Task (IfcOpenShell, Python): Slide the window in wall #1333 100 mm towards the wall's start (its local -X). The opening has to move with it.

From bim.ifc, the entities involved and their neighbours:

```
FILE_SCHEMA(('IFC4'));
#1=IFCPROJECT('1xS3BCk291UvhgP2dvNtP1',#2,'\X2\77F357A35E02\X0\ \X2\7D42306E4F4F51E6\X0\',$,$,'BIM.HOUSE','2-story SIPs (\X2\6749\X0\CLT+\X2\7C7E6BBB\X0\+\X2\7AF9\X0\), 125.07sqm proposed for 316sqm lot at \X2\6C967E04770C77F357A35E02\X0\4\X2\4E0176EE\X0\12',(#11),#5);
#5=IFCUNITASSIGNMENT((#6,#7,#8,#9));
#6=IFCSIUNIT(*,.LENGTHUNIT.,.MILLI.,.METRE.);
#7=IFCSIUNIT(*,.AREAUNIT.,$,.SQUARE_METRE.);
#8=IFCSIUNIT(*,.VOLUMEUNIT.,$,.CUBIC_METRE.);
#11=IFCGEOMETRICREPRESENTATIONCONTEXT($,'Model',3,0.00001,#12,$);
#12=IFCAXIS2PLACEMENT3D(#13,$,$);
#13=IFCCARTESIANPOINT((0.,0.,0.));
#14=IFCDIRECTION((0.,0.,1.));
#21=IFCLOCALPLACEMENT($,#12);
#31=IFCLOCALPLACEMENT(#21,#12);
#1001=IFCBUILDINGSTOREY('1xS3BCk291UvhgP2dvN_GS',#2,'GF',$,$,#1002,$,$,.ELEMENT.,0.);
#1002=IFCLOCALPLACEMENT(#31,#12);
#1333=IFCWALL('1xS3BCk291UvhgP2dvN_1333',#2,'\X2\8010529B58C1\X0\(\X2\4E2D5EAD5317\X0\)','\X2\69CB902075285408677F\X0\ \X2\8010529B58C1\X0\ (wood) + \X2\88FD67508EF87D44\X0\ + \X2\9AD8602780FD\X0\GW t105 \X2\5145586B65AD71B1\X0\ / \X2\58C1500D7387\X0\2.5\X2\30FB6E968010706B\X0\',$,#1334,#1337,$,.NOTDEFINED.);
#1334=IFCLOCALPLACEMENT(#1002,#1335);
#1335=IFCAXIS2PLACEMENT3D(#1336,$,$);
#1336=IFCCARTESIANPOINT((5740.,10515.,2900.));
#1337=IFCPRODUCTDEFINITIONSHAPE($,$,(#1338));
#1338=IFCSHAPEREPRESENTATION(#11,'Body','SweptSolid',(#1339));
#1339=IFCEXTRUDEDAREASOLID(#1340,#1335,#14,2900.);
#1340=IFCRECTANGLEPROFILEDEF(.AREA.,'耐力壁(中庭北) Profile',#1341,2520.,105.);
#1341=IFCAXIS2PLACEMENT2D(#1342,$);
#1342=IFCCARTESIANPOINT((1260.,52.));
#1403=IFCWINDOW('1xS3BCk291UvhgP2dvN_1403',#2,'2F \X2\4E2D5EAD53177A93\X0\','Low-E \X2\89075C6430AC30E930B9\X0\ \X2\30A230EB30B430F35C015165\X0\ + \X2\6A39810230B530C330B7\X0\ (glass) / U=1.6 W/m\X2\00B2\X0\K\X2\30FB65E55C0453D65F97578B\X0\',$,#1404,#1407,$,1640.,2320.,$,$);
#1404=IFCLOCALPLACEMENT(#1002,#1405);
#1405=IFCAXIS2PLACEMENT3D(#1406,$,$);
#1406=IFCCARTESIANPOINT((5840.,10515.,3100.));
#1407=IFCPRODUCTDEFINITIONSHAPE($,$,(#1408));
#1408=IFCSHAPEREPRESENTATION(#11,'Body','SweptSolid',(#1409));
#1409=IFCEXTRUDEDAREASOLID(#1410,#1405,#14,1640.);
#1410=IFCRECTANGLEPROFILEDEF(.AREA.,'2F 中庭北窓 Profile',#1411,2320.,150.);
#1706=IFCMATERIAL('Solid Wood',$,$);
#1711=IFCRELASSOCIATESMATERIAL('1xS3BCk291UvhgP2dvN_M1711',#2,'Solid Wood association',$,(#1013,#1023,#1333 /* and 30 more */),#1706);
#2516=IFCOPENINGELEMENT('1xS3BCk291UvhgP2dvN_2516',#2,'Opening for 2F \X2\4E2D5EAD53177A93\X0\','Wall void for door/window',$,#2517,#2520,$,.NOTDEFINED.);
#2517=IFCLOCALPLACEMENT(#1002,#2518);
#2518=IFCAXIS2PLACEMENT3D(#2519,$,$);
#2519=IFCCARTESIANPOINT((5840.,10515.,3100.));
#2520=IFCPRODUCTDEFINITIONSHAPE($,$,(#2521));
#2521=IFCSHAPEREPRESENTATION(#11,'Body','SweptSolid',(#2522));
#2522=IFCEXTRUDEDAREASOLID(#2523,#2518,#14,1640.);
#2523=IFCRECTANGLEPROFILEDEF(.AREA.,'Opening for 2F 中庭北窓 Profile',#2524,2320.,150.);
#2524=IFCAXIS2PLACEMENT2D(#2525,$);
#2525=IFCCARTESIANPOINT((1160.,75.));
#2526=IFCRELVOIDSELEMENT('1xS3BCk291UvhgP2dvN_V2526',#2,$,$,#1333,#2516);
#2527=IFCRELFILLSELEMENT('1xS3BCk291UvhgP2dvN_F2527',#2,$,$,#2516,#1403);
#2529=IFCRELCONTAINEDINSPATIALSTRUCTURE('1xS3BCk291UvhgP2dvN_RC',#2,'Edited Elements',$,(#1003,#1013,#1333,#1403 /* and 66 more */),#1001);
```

```python
import ifcopenshell
import ifcopenshell.api.geometry
import ifcopenshell.util.placement
import ifcopenshell.util.unit

model = ifcopenshell.open("bim.ifc")
unit_scale = ifcopenshell.util.unit.calculate_unit_scale(model)

window = model.by_id(1403)
opening = window.FillsVoids[0].RelatingOpeningElement
wall = opening.VoidsElements[0].RelatingBuildingElement

wall_matrix = ifcopenshell.util.placement.get_local_placement(wall.ObjectPlacement)
shift = wall_matrix[:3, 0] * -0.1 / unit_scale
before = ifcopenshell.util.placement.get_local_placement(window.ObjectPlacement)[:3, 3].copy()

# The window is not placed relative to its opening, so move both.
for product in (opening, window):
    matrix = ifcopenshell.util.placement.get_local_placement(product.ObjectPlacement)
    matrix[:3, 3] += shift
    ifcopenshell.api.geometry.edit_object_placement(model, product=product, matrix=matrix, is_si=False)

after = ifcopenshell.util.placement.get_local_placement(window.ObjectPlacement)[:3, 3]
print("window moved by", (after - before).round(3) + 0.0)

model.write("bim_rev.ifc")
```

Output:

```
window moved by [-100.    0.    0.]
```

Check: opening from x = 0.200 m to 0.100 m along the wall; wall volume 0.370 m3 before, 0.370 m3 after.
